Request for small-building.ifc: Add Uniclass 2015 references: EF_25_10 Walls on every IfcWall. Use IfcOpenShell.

First a look at what the model holds.

```python
import ifcopenshell

model = ifcopenshell.open("small-building.ifc")
print(model.schema)
print("classifications:", [c.Name for c in model.by_type("IfcClassification")])
for ifc_class in ("IfcDoor", "IfcRoof", "IfcStair", "IfcWall", "IfcWindow"):
    print(ifc_class, len(model.by_type(ifc_class)))
```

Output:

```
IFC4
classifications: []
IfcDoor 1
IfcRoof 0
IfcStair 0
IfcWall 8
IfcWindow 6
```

```python
import ifcopenshell
import ifcopenshell.api.classification

model = ifcopenshell.open("small-building.ifc")

system = ifcopenshell.api.classification.add_classification(model, classification="Uniclass 2015")

codes = {
    "IfcWall": ("EF_25_10", "Walls"),
}
for ifc_class, (code, name) in codes.items():
    products = model.by_type(ifc_class)
    ifcopenshell.api.classification.add_reference(
        model, products=products, classification=system, identification=code, name=name
    )
    print(code, len(products))

model.write("small-building_rev.ifc")
```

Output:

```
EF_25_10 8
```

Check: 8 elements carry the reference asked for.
